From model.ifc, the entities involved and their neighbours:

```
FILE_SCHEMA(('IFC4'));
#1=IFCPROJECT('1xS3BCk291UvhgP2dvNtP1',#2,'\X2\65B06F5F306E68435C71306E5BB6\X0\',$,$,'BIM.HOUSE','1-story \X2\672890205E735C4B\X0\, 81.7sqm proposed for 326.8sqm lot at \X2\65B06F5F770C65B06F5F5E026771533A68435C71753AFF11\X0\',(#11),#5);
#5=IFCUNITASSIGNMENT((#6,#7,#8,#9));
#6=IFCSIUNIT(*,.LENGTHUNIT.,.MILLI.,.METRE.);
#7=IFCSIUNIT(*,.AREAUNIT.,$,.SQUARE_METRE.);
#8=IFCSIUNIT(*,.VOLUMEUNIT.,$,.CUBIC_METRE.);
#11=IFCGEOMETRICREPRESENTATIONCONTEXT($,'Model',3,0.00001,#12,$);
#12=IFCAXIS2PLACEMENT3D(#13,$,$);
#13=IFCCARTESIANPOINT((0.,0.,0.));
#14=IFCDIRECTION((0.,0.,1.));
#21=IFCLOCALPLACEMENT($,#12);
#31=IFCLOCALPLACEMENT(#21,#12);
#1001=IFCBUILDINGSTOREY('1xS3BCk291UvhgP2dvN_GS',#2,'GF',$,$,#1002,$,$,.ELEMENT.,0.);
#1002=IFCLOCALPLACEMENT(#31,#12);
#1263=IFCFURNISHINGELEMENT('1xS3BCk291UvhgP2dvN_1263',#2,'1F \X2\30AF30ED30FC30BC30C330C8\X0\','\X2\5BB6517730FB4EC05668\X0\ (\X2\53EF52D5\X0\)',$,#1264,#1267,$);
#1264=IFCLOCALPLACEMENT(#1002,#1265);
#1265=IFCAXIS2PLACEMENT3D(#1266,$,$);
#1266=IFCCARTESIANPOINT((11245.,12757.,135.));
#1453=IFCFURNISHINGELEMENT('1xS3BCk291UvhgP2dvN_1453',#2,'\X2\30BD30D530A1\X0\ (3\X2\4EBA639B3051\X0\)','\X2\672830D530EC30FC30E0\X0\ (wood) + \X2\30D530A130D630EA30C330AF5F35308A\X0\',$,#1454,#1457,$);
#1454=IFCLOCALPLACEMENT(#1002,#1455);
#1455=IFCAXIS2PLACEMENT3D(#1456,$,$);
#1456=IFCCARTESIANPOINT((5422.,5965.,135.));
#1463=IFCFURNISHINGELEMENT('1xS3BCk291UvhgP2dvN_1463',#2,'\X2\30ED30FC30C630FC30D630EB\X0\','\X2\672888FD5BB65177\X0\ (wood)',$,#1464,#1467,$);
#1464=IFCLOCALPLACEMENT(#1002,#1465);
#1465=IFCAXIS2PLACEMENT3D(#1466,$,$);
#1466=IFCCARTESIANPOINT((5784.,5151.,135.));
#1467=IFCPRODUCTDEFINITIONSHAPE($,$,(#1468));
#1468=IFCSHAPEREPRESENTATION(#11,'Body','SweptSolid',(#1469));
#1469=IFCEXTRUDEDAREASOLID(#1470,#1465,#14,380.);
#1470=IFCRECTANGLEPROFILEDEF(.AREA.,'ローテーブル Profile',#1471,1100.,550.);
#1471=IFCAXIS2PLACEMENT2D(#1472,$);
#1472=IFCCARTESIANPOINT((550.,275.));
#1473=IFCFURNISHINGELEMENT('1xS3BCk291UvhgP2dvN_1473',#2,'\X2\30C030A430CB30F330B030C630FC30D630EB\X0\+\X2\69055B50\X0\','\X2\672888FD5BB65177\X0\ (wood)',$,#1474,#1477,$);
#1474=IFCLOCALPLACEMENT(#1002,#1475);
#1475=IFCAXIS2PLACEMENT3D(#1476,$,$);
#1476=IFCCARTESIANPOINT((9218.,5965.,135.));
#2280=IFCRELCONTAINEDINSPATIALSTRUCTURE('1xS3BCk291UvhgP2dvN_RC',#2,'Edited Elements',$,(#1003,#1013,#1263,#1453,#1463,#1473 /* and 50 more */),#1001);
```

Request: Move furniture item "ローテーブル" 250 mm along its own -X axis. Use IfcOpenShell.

```python
import ifcopenshell
import ifcopenshell.api.geometry
import ifcopenshell.util.placement
import ifcopenshell.util.unit

model = ifcopenshell.open("model.ifc")
unit_scale = ifcopenshell.util.unit.calculate_unit_scale(model)

item = model.by_guid("1xS3BCk291UvhgP2dvN_1463")
matrix = ifcopenshell.util.placement.get_local_placement(item.ObjectPlacement)
matrix[:3, 3] -= matrix[:3, 0] * 0.25 / unit_scale
ifcopenshell.api.geometry.edit_object_placement(model, product=item, matrix=matrix, is_si=False)

print(ifcopenshell.util.placement.get_local_placement(item.ObjectPlacement).round(3) + 0.0)

model.write("model_edited.ifc")
```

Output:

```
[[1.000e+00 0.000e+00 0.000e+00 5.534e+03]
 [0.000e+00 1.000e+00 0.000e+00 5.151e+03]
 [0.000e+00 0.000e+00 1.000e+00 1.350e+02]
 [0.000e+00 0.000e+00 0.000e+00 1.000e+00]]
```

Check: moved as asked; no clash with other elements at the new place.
